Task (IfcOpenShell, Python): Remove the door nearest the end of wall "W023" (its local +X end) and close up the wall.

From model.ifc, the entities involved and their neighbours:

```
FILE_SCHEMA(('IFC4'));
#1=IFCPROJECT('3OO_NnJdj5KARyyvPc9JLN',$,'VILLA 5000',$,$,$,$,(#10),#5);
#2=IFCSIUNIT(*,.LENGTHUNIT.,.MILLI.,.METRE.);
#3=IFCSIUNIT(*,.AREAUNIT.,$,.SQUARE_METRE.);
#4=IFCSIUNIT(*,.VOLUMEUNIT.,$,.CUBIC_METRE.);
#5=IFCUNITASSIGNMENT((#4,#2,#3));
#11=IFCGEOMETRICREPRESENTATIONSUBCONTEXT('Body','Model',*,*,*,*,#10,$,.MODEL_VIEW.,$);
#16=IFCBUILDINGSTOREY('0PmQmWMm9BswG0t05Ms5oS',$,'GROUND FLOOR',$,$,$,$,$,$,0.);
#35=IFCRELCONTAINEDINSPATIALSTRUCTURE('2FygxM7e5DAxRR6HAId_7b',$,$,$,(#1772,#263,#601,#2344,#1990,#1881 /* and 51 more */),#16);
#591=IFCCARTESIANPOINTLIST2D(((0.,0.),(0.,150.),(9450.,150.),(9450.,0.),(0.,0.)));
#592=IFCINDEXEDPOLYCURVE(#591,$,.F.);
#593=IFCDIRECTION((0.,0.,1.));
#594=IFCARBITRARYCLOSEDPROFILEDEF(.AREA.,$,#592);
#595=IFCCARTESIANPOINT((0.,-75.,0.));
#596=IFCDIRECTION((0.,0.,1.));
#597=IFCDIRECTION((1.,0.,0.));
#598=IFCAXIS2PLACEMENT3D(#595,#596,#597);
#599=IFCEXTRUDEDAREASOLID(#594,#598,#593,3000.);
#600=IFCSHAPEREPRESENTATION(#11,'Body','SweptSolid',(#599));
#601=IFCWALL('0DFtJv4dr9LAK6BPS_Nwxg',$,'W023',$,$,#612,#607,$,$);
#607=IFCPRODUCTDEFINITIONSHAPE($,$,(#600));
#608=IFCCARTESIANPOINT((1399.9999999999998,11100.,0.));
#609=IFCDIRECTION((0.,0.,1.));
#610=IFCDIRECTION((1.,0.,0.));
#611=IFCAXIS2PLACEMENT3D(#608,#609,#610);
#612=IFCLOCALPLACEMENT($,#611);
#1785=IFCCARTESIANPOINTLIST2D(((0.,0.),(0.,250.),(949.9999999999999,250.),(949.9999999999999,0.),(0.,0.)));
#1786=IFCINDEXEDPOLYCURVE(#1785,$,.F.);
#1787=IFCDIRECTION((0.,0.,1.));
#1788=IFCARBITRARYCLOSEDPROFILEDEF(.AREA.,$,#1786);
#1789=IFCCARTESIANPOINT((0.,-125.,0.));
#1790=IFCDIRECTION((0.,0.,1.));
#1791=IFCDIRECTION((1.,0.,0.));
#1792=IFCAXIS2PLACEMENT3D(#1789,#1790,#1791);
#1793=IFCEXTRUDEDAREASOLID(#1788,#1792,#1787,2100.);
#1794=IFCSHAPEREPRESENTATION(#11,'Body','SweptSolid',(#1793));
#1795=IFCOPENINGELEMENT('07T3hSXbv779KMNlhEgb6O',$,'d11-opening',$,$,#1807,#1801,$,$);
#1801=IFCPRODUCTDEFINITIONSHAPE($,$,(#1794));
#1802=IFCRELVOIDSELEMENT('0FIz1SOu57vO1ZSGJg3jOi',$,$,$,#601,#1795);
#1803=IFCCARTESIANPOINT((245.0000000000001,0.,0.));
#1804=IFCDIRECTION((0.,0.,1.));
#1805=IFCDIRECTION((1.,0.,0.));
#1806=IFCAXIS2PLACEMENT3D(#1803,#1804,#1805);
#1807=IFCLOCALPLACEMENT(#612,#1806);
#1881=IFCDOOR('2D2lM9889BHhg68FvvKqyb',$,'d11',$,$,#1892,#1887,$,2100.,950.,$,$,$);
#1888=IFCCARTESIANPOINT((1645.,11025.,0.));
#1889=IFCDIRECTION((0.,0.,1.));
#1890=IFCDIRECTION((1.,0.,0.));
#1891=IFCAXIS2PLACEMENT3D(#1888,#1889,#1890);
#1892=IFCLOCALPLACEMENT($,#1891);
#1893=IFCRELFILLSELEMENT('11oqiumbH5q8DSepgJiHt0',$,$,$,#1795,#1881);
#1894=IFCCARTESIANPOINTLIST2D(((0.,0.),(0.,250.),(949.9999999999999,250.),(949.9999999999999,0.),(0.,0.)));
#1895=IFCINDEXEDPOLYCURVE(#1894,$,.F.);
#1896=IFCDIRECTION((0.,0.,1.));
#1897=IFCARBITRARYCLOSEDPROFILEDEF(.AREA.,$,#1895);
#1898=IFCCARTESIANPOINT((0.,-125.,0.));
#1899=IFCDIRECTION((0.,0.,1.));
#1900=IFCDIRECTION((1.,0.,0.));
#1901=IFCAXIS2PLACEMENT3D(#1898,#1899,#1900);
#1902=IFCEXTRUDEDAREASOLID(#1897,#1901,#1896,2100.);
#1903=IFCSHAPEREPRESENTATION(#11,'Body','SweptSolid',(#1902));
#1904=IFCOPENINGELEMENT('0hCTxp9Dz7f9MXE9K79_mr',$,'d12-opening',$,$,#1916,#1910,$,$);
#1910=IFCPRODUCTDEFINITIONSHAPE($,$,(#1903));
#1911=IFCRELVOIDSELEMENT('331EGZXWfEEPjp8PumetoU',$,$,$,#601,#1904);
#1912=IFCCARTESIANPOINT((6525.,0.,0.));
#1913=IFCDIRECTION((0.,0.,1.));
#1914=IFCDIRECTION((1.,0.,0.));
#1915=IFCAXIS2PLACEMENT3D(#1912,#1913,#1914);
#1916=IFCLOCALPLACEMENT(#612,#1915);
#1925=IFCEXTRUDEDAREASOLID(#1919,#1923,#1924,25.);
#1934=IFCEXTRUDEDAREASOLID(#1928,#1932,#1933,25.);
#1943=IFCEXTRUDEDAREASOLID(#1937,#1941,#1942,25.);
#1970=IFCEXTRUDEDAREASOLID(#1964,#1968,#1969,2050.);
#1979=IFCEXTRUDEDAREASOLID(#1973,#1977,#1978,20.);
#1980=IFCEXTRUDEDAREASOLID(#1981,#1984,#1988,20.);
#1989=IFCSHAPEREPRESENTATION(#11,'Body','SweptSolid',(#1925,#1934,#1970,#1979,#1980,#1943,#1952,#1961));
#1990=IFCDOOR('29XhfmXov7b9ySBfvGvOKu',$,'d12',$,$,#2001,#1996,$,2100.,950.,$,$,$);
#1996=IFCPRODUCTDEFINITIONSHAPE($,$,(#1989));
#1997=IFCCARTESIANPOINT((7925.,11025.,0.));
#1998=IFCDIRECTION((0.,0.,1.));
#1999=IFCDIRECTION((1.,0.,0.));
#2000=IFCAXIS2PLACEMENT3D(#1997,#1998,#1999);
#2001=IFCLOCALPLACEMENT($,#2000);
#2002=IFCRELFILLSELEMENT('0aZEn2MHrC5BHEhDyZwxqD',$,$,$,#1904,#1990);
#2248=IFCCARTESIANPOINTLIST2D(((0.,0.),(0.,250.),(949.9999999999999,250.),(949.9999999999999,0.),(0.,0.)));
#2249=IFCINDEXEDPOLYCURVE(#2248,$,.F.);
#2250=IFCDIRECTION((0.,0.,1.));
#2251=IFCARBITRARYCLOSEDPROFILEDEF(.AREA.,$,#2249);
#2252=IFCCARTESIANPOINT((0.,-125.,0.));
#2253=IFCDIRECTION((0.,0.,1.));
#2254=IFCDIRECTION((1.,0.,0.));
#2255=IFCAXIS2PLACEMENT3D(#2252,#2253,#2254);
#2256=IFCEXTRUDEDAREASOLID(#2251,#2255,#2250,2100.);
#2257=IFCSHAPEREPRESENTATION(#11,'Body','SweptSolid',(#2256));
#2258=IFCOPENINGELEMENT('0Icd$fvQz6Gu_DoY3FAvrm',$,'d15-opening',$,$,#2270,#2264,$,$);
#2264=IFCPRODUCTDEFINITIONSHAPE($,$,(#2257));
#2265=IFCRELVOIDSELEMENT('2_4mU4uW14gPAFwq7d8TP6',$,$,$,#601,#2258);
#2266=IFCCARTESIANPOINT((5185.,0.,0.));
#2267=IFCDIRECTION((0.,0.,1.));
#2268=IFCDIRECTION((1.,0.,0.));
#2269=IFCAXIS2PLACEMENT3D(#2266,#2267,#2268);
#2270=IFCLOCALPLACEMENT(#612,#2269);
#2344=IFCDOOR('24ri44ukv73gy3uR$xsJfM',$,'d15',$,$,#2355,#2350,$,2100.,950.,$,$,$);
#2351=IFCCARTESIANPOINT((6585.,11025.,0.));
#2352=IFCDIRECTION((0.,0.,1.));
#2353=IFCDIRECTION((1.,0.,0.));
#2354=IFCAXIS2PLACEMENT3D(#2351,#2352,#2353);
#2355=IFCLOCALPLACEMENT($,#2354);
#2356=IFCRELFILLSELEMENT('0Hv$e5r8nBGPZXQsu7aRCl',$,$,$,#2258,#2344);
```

```python
import ifcopenshell
import ifcopenshell.api.feature
import ifcopenshell.api.root
import ifcopenshell.geom
import ifcopenshell.util.shape

model = ifcopenshell.open("model.ifc")
settings = ifcopenshell.geom.settings()


def volume(element):
    """Net volume in cubic metres, openings subtracted."""
    shape = ifcopenshell.geom.create_shape(settings, element)
    return ifcopenshell.util.shape.get_volume(shape.geometry)


door = model.by_guid("29XhfmXov7b9ySBfvGvOKu")
opening = door.FillsVoids[0].RelatingOpeningElement
wall = opening.VoidsElements[0].RelatingBuildingElement
before = volume(wall)

ifcopenshell.api.root.remove_product(model, product=door)
ifcopenshell.api.feature.remove_feature(model, feature=opening)

after = volume(wall)

print(f"wall volume {before:.3f} -> {after:.3f} m3")

model.write("model_rev.ifc")
```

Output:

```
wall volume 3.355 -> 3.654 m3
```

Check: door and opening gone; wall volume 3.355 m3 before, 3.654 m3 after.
